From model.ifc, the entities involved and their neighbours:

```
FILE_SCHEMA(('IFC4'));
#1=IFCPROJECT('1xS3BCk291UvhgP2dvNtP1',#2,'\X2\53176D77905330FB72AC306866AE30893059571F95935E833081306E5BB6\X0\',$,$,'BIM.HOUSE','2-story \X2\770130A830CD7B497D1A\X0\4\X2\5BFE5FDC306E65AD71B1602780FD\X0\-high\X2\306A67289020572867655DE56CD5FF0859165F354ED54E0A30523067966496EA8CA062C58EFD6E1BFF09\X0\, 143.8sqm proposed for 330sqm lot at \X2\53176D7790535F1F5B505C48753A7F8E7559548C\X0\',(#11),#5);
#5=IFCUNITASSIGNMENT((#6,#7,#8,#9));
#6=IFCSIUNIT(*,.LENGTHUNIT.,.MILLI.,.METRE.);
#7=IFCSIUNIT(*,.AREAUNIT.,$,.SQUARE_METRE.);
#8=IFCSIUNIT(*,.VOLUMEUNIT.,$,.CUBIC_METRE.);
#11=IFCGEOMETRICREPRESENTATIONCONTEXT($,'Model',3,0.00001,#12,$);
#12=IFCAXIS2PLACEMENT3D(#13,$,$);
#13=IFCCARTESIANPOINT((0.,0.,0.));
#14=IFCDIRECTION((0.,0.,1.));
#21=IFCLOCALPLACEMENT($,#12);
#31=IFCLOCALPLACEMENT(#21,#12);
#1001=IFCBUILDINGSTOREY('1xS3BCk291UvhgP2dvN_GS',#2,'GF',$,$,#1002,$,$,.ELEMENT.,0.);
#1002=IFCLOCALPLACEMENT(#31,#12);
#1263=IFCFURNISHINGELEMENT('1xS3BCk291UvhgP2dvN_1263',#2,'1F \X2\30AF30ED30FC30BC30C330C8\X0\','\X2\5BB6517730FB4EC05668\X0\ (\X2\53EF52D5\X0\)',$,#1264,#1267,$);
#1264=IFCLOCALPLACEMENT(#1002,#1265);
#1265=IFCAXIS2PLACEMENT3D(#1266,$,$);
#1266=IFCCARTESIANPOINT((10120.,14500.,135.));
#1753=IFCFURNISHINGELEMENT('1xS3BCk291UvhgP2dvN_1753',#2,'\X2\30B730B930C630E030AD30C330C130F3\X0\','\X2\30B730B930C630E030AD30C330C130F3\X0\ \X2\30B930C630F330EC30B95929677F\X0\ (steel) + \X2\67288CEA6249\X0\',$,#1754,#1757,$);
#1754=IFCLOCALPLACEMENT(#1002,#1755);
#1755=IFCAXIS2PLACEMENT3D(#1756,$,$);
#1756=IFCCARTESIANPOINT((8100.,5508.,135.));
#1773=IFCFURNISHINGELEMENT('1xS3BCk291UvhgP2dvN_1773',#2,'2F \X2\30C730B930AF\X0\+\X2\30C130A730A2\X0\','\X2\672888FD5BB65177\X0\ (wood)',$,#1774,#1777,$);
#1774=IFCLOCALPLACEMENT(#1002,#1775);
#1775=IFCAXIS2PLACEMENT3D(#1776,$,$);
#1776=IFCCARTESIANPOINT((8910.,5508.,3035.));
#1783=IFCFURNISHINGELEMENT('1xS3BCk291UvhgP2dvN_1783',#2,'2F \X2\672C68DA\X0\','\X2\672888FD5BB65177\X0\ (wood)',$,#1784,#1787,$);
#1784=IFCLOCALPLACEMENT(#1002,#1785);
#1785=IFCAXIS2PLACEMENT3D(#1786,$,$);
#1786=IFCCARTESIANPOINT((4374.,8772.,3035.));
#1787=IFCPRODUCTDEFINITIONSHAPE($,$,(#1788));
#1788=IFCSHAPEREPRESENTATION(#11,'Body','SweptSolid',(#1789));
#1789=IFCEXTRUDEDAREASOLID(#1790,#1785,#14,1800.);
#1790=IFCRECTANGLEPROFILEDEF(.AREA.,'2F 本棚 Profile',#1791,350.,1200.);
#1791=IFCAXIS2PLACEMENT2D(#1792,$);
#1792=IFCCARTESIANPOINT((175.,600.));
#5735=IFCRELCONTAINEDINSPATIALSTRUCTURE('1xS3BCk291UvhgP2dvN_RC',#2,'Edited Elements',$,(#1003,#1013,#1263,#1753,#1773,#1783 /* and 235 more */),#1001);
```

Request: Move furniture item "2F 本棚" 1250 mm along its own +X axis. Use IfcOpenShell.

```python
import ifcopenshell
import ifcopenshell.api.geometry
import ifcopenshell.util.placement
import ifcopenshell.util.unit

model = ifcopenshell.open("model.ifc")
unit_scale = ifcopenshell.util.unit.calculate_unit_scale(model)

item = model.by_guid("1xS3BCk291UvhgP2dvN_1783")
matrix = ifcopenshell.util.placement.get_local_placement(item.ObjectPlacement)
matrix[:3, 3] += matrix[:3, 0] * 1.25 / unit_scale
ifcopenshell.api.geometry.edit_object_placement(model, product=item, matrix=matrix, is_si=False)

print(ifcopenshell.util.placement.get_local_placement(item.ObjectPlacement).round(3) + 0.0)

model.write("model_rev.ifc")
```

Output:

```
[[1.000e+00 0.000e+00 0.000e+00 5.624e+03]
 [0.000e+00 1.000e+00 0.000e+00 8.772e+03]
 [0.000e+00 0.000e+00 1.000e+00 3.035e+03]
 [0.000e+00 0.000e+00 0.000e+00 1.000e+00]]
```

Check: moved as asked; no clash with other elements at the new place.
